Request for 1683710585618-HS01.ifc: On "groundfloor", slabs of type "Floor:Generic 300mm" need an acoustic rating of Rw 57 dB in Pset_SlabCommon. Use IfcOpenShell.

First a look at what the model holds.

```python
import ifcopenshell
import ifcopenshell.util.element

model = ifcopenshell.open("1683710585618-HS01.ifc")
print(model.schema)
storey = next(s for s in model.by_type("IfcBuildingStorey") if s.Name == "groundfloor")
slabs = [e for e in ifcopenshell.util.element.get_decomposition(storey) if e.is_a("IfcSlab")]
seen = {}
for e in slabs:
    element_type = ifcopenshell.util.element.get_type(e)
    key = (element_type.Name if element_type != e and element_type else None, ifcopenshell.util.element.get_pset(e, "Pset_SlabCommon", "AcousticRating"))
    seen[key] = seen.get(key, 0) + 1
for (name, value), count in sorted(seen.items(), key=str):
    print(count, "x", name, "|", value)
```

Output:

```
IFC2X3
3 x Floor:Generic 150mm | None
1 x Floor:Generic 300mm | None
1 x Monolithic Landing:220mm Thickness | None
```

```python
import ifcopenshell
import ifcopenshell.api.pset
import ifcopenshell.util.element

model = ifcopenshell.open("1683710585618-HS01.ifc")

storey = next(s for s in model.by_type("IfcBuildingStorey") if s.Name == "groundfloor")
slabs = [e for e in ifcopenshell.util.element.get_decomposition(storey) if e.is_a("IfcSlab")]

count = 0
for e in slabs:
    element_type = ifcopenshell.util.element.get_type(e)
    if element_type in (None, e) or element_type.Name != "Floor:Generic 300mm":
        continue
    # add_pset returns the element's existing set when there is one.
    pset = ifcopenshell.api.pset.add_pset(model, product=e, name="Pset_SlabCommon")
    ifcopenshell.api.pset.edit_pset(model, pset=pset, properties={"AcousticRating": "Rw 57 dB"})
    count += 1

print(count, "slabs updated")

model.write("1683710585618-HS01_v2.ifc")
```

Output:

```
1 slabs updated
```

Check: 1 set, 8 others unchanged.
